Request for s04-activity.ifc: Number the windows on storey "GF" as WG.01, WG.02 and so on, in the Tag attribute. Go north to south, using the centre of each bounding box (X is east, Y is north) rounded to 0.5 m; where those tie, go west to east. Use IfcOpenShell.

First a look at what the model holds.

```python
import ifcopenshell
import ifcopenshell.util.element
import ifcopenshell.util.placement

model = ifcopenshell.open("s04-activity.ifc")
print(model.schema)
storey = next(s for s in model.by_type("IfcBuildingStorey") if s.Name == "GF")
windows = [e for e in ifcopenshell.util.element.get_decomposition(storey) if e.is_a("IfcWindow")]
for e in sorted(windows, key=lambda e: e.id()):
    origin = ifcopenshell.util.placement.get_local_placement(e.ObjectPlacement)[:3, 3]
    print(e.id(), e.Tag, e.Name, origin.round(2) + 0.0, sep=" | ")
```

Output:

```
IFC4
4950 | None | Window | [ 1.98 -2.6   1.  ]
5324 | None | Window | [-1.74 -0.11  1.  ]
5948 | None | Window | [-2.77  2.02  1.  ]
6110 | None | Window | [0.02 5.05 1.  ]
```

```python
import ifcopenshell
import ifcopenshell.geom
import ifcopenshell.util.element
import ifcopenshell.util.shape

model = ifcopenshell.open("s04-activity.ifc")
settings = ifcopenshell.geom.settings()
settings.set("use-world-coords", True)


def centre(element):
    shape = ifcopenshell.geom.create_shape(settings, element)
    return ifcopenshell.util.shape.get_bbox_centroid(shape.geometry)


storey = next(s for s in model.by_type("IfcBuildingStorey") if s.Name == "GF")
windows = [e for e in ifcopenshell.util.element.get_decomposition(storey) if e.is_a("IfcWindow")]

# Insertion points can sit at a corner or the storey origin, so sort by the geometry (in metres).
centres = {e: centre(e) for e in windows}
windows.sort(key=lambda e: (-round(centres[e][1] / 0.5), centres[e][0]))

for i, e in enumerate(windows, start=1):
    number = f"WG.{i:02d}"
    e.Tag = number
    print(e.id(), number)

model.write("s04-activity_updated.ifc")
```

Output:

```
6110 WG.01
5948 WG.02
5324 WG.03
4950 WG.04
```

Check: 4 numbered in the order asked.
